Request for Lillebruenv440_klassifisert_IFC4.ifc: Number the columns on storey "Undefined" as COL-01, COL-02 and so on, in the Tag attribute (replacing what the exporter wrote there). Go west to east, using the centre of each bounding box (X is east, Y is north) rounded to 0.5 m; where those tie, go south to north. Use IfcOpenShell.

First a look at what the model holds.

```python
import ifcopenshell
import ifcopenshell.util.element
import ifcopenshell.util.placement

model = ifcopenshell.open("Lillebruenv440_klassifisert_IFC4.ifc")
print(model.schema)
storey = next(s for s in model.by_type("IfcBuildingStorey") if s.Name == "Undefined")
columns = [e for e in ifcopenshell.util.element.get_decomposition(storey) if e.is_a("IfcColumn")]
for e in sorted(columns, key=lambda e: e.id()):
    origin = ifcopenshell.util.placement.get_local_placement(e.ObjectPlacement)[:3, 3]
    print(e.id(), e.Tag, e.Name, origin.round(2) + 0.0, sep=" | ")
```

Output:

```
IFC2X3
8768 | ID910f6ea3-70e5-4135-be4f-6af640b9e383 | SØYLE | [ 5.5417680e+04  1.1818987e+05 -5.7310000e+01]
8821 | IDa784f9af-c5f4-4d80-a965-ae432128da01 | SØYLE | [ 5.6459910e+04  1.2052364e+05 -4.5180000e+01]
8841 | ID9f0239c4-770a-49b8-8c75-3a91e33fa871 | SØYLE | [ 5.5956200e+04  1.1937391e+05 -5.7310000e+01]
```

```python
import ifcopenshell
import ifcopenshell.geom
import ifcopenshell.util.element
import ifcopenshell.util.shape

model = ifcopenshell.open("Lillebruenv440_klassifisert_IFC4.ifc")
settings = ifcopenshell.geom.settings()
settings.set("use-world-coords", True)


def centre(element):
    shape = ifcopenshell.geom.create_shape(settings, element)
    return ifcopenshell.util.shape.get_bbox_centroid(shape.geometry)


storey = next(s for s in model.by_type("IfcBuildingStorey") if s.Name == "Undefined")
columns = [e for e in ifcopenshell.util.element.get_decomposition(storey) if e.is_a("IfcColumn")]

# Insertion points can sit at a corner or the storey origin, so sort by the geometry (in metres).
centres = {e: centre(e) for e in columns}
columns.sort(key=lambda e: (round(centres[e][0] / 0.5), centres[e][1]))

for i, e in enumerate(columns, start=1):
    number = f"COL-{i:02d}"
    e.Tag = number
    print(e.id(), number)

model.write("Lillebruenv440_klassifisert_IFC4_v2.ifc")
```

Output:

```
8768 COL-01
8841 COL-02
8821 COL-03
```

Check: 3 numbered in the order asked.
